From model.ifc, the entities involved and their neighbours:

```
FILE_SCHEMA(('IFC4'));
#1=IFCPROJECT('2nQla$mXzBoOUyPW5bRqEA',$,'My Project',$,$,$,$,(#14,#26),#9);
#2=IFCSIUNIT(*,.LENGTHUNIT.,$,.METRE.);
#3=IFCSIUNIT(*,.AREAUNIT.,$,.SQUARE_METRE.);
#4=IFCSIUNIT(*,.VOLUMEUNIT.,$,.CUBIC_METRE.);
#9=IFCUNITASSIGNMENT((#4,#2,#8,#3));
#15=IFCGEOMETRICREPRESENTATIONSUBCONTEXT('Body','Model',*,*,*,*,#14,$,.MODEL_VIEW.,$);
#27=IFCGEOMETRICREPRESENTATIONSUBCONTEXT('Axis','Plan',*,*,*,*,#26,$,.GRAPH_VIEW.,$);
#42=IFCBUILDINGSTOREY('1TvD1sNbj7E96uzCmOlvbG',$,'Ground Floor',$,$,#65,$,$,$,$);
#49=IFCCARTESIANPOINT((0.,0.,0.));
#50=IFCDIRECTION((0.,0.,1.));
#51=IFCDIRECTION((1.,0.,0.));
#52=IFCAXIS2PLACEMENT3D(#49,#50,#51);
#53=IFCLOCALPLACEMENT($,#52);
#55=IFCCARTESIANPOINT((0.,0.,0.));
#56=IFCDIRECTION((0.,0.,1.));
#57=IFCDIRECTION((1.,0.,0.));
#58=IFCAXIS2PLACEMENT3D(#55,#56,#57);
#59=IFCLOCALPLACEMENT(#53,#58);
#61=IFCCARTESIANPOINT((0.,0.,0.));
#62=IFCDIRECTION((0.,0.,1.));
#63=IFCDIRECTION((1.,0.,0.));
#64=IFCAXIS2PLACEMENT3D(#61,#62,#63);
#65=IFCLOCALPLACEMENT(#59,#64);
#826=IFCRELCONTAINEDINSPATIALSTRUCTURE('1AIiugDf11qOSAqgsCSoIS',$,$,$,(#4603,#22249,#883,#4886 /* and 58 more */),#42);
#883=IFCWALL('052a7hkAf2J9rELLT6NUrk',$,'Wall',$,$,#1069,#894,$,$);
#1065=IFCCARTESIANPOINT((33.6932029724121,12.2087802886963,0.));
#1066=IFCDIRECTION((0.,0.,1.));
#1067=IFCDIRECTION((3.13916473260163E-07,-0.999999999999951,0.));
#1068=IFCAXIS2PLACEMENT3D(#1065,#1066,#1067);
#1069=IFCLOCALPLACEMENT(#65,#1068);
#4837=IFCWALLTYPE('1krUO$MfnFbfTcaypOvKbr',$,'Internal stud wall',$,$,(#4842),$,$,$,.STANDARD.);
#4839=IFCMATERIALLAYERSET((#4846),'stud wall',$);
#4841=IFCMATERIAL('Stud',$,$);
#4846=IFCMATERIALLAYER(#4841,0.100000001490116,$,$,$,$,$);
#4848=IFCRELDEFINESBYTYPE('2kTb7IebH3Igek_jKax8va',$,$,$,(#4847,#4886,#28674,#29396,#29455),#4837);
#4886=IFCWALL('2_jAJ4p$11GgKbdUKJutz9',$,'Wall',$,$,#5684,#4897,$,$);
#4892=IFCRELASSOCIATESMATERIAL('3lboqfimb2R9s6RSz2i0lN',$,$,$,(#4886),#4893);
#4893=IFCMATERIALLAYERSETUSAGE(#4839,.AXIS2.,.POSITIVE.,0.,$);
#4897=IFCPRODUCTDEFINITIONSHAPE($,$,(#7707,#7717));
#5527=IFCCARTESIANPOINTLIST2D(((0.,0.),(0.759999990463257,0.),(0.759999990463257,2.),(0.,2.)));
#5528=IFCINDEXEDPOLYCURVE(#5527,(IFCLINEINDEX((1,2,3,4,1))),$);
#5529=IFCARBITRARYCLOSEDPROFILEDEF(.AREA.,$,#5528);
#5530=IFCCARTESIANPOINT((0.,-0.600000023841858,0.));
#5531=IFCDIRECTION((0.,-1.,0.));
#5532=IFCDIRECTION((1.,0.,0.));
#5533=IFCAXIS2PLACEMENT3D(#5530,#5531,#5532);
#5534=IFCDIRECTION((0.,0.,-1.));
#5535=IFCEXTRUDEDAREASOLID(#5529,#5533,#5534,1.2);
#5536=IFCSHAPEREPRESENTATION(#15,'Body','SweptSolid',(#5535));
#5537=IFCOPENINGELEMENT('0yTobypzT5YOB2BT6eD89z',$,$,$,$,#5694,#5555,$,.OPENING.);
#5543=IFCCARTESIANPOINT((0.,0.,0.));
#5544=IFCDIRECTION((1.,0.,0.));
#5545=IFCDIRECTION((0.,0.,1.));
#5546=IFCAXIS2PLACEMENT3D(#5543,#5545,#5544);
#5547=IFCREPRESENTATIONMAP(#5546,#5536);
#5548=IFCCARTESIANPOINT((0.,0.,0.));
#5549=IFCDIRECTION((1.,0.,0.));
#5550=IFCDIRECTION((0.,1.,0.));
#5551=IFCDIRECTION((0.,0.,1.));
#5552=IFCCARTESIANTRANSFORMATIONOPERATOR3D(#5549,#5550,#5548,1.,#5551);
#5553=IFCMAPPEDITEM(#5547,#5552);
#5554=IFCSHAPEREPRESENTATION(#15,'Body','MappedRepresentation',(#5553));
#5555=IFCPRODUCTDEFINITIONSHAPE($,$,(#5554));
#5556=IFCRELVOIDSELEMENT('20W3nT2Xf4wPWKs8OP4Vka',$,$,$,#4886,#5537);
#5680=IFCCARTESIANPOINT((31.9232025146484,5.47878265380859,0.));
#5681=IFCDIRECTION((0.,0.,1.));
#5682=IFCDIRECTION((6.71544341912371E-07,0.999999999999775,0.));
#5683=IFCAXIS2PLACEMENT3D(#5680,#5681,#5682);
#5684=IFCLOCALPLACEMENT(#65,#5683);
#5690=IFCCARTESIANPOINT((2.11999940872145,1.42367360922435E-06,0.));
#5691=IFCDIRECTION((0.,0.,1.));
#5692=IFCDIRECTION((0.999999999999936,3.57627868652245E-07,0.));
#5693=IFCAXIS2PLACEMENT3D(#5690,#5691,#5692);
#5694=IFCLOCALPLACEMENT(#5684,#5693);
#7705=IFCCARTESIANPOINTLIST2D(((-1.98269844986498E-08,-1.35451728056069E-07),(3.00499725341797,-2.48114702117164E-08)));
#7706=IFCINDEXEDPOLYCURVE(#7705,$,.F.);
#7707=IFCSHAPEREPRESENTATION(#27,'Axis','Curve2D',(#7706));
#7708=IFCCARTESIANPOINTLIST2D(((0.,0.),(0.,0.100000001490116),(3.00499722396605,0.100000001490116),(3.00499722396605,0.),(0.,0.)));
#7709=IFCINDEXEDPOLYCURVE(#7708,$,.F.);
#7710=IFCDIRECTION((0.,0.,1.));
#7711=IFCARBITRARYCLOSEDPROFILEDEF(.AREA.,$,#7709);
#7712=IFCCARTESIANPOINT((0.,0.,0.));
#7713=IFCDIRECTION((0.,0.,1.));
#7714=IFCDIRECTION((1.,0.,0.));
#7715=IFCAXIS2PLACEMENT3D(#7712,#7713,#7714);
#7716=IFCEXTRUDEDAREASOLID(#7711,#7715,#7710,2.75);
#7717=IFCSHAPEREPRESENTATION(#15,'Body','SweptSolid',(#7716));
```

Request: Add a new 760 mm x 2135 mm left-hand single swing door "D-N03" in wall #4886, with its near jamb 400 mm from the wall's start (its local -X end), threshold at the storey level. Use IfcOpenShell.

```python
import numpy as np
import ifcopenshell
import ifcopenshell.api.feature
import ifcopenshell.api.geometry
import ifcopenshell.api.root
import ifcopenshell.api.spatial
import ifcopenshell.geom
import ifcopenshell.util.element
import ifcopenshell.util.placement
import ifcopenshell.util.representation
import ifcopenshell.util.shape
import ifcopenshell.util.unit

model = ifcopenshell.open("model.ifc")
unit_scale = ifcopenshell.util.unit.calculate_unit_scale(model)
settings = ifcopenshell.geom.settings()


def volume(element):
    """Net volume in cubic metres, openings subtracted."""
    shape = ifcopenshell.geom.create_shape(settings, element)
    return ifcopenshell.util.shape.get_volume(shape.geometry)


wall = model.by_guid("2_jAJ4p$11GgKbdUKJutz9")
storey = ifcopenshell.util.element.get_container(wall, ifc_class="IfcBuildingStorey")
context = ifcopenshell.util.representation.get_context(model, "Model", "Body", "MODEL_VIEW")
before = volume(wall)

width, height, from_end, sill = 0.76, 2.135, 0.4, 0.0  # metres

# The wall runs along its own X axis, and the end named is its -X end.
wall_shape = ifcopenshell.geom.create_shape(settings, wall)
x, y, z = ifcopenshell.util.shape.get_vertices(wall_shape.geometry).T
start = x.min() + from_end
face, thickness = float(y.min()), float(y.max() - y.min())
wall_matrix = ifcopenshell.util.placement.get_local_placement(wall.ObjectPlacement)
level = ifcopenshell.util.placement.get_local_placement(storey.ObjectPlacement)[2, 3]


def in_wall(x, y):
    """Placement at x, y metres in the wall's axes, at sill height."""
    matrix = wall_matrix.copy()
    matrix[:, 3] = wall_matrix @ np.array([x / unit_scale, y / unit_scale, 0.0, 1.0])
    matrix[2, 3] = level + sill / unit_scale
    return matrix


# Opening: a box that overshoots both wall faces by 50 mm.
opening = ifcopenshell.api.root.create_entity(model, ifc_class="IfcOpeningElement", predefined_type="OPENING")
box = ifcopenshell.api.geometry.add_wall_representation(
    model, context=context, length=width, height=height, thickness=thickness + 0.1
)
ifcopenshell.api.geometry.assign_representation(model, product=opening, representation=box)
ifcopenshell.api.geometry.edit_object_placement(model, product=opening, matrix=in_wall(start, face - 0.05), is_si=False)
ifcopenshell.api.feature.add_feature(model, feature=opening, element=wall)

door = ifcopenshell.api.root.create_entity(model, ifc_class="IfcDoor", name="D-N03", predefined_type="DOOR")
door.OverallWidth, door.OverallHeight = width / unit_scale, height / unit_scale
door.OperationType = "SINGLE_SWING_LEFT"
body = ifcopenshell.api.geometry.add_door_representation(
    model,
    context=context,
    overall_width=door.OverallWidth,
    overall_height=door.OverallHeight,
    operation_type="SINGLE_SWING_LEFT",
    lining_properties={"LiningDepth": thickness / unit_scale, "ThresholdDepth": thickness / unit_scale},
)
ifcopenshell.api.geometry.assign_representation(model, product=door, representation=body)
ifcopenshell.api.spatial.assign_container(model, products=[door], relating_structure=storey)
ifcopenshell.api.feature.add_filling(model, opening=opening, element=door)

# The lining spans the wall, so the door starts at the wall face.
ifcopenshell.api.geometry.edit_object_placement(model, product=door, matrix=in_wall(start, face), is_si=False)

after = volume(wall)

print(f"wall volume {before:.3f} -> {after:.3f} m3")

model.write("model_v2.ifc")
```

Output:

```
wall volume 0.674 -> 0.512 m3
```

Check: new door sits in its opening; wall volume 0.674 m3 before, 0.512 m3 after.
